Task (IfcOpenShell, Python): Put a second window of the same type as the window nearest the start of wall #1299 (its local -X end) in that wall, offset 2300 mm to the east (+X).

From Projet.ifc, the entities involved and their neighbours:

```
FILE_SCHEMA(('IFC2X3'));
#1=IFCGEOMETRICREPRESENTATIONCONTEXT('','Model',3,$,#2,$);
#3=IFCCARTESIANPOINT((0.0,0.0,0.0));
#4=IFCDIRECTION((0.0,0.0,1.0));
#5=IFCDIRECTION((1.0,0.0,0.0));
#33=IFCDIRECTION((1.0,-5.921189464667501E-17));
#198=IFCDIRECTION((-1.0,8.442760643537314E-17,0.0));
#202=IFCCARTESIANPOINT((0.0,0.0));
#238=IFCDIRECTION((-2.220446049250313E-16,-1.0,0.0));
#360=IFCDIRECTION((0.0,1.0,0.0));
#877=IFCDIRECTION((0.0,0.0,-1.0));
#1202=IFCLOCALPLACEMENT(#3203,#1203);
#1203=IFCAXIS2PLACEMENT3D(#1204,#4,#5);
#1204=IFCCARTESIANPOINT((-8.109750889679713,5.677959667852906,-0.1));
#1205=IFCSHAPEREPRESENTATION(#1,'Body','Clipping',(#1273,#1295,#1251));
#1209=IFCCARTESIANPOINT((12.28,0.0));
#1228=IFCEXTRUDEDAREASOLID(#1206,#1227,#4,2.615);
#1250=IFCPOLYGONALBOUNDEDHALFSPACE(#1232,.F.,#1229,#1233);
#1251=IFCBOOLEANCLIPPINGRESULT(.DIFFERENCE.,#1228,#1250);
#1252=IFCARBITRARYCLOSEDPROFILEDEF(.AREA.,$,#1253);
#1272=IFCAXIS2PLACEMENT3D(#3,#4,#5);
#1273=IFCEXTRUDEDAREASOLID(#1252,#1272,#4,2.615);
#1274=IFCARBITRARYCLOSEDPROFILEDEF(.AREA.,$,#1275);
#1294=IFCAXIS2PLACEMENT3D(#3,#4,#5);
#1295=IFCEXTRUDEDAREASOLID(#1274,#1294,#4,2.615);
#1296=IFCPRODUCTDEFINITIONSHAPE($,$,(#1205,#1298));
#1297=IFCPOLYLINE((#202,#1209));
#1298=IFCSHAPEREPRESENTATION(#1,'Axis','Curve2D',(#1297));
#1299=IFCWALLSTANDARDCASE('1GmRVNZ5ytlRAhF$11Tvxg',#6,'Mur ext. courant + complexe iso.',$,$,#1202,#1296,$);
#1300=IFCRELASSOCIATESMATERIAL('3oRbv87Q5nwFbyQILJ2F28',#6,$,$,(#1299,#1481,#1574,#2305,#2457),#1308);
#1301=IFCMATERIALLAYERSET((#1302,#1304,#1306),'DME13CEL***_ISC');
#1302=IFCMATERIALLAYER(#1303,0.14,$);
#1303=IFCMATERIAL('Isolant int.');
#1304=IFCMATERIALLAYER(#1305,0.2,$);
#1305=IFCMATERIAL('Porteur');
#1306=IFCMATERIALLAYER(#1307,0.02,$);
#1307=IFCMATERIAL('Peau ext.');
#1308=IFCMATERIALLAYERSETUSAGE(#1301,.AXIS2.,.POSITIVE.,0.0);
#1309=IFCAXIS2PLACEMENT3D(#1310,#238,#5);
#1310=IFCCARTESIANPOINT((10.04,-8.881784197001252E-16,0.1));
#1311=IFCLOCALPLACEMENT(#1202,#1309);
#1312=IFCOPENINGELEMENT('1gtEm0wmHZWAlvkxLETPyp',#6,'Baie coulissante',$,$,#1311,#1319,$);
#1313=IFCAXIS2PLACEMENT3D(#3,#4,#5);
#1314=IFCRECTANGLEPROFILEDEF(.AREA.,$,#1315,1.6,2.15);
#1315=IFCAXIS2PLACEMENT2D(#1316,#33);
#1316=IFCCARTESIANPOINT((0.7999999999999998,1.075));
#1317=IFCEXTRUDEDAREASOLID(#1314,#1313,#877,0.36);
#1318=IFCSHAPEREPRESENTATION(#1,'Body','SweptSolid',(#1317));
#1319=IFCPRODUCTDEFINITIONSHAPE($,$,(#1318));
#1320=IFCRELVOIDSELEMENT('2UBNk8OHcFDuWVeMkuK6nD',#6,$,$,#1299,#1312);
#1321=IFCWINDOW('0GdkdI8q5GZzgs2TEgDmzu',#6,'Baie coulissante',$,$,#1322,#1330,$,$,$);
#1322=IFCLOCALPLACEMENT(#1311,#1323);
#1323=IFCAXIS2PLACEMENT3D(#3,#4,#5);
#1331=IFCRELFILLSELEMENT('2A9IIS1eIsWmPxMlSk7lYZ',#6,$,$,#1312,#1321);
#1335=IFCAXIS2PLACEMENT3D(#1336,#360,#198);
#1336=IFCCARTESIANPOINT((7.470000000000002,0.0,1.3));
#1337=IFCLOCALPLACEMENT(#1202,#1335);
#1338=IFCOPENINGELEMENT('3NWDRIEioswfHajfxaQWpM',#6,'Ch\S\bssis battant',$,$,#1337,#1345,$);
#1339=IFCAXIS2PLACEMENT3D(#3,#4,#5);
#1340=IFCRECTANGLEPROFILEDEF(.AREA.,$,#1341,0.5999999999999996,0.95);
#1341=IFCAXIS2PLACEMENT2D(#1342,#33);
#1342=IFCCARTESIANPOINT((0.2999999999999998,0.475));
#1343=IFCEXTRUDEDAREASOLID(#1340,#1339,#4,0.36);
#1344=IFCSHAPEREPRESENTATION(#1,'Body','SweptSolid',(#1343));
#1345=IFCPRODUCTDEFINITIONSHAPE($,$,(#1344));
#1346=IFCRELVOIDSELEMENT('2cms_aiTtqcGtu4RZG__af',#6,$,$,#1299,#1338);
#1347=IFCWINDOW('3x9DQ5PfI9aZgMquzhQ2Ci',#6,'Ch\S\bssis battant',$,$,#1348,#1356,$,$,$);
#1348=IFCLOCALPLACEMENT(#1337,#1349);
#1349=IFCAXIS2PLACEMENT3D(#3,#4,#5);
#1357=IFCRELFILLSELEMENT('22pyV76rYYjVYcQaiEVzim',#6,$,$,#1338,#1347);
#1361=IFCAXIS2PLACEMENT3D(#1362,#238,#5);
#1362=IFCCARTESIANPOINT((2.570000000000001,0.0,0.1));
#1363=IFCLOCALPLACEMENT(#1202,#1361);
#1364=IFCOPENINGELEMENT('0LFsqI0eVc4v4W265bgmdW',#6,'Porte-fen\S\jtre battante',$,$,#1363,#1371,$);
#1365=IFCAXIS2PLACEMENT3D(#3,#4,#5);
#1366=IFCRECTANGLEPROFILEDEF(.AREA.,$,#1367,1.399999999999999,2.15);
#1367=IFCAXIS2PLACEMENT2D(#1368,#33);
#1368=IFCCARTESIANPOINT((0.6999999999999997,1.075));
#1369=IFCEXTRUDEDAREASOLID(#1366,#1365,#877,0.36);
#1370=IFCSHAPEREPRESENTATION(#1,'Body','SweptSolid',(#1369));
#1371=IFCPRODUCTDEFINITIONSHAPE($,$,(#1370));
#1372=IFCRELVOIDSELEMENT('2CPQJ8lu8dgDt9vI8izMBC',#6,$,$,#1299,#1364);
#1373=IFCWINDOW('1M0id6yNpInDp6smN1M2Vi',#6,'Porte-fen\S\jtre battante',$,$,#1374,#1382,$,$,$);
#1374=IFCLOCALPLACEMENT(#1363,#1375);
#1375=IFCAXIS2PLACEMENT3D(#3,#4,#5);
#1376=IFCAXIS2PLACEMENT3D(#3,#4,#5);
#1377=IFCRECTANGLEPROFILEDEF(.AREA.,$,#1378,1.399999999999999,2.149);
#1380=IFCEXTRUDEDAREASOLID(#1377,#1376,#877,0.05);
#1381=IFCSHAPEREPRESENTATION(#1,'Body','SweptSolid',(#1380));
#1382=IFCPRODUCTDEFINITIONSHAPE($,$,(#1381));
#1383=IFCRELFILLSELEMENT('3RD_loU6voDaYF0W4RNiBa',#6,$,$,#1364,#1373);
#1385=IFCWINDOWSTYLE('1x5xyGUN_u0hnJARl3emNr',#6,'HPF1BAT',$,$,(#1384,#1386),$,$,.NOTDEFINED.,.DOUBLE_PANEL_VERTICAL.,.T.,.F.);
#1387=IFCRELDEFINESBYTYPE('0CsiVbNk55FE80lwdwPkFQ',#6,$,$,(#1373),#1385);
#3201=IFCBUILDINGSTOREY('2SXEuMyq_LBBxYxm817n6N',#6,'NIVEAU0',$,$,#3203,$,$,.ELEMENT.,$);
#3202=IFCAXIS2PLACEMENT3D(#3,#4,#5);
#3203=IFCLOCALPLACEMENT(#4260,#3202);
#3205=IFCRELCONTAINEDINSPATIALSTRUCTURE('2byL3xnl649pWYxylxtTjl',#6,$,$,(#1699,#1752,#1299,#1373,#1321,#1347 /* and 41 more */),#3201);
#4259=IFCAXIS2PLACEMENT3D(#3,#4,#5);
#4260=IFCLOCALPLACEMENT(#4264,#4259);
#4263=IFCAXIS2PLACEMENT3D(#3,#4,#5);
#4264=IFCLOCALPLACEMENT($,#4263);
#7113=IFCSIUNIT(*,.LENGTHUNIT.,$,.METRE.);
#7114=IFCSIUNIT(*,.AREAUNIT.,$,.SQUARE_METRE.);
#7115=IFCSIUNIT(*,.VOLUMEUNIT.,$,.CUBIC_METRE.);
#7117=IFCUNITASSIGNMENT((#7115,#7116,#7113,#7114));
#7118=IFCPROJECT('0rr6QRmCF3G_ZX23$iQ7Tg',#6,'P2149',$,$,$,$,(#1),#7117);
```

```python
import ifcopenshell
import ifcopenshell.api.feature
import ifcopenshell.api.geometry
import ifcopenshell.api.root
import ifcopenshell.geom
import ifcopenshell.util.element
import ifcopenshell.util.placement
import ifcopenshell.util.shape

model = ifcopenshell.open("Projet.ifc")
settings = ifcopenshell.geom.settings()


def volume(element):
    """Net volume in cubic metres, openings subtracted."""
    shape = ifcopenshell.geom.create_shape(settings, element)
    return ifcopenshell.util.shape.get_volume(shape.geometry)


window = model.by_guid("1M0id6yNpInDp6smN1M2Vi")
opening = window.FillsVoids[0].RelatingOpeningElement
wall = opening.VoidsElements[0].RelatingBuildingElement
before = volume(wall)
shift = ifcopenshell.util.placement.get_local_placement(wall.ObjectPlacement)[:3, 0] * 2.3

# copy_class copies the void relationship, type, container and properties, but no geometry.
new_opening = ifcopenshell.api.root.copy_class(model, product=opening)
new_opening.Representation = ifcopenshell.util.element.copy_deep(
    model, opening.Representation, exclude=["IfcGeometricRepresentationContext", "IfcRepresentationMap"]
)
new_window = ifcopenshell.api.root.copy_class(model, product=window)
new_window.Representation = ifcopenshell.util.element.copy_deep(
    model, window.Representation, exclude=["IfcGeometricRepresentationContext", "IfcRepresentationMap"]
)
fills = ifcopenshell.api.feature.add_filling(model, opening=new_opening, element=new_window)
fills.OwnerHistory = new_window.OwnerHistory  # required in IFC2X3

for old, new in ((opening, new_opening), (window, new_window)):
    matrix = ifcopenshell.util.placement.get_local_placement(old.ObjectPlacement)
    matrix[:3, 3] += shift
    ifcopenshell.api.geometry.edit_object_placement(model, product=new, matrix=matrix, is_si=False)

after = volume(wall)

print(f"wall volume {before:.3f} -> {after:.3f} m3")

model.write("Projet_v2.ifc")
```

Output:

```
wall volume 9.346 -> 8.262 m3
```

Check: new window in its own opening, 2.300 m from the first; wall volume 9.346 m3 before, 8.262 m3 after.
